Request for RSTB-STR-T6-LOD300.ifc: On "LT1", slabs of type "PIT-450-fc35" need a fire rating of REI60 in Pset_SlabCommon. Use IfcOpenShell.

First a look at what the model holds.

```python
import ifcopenshell
import ifcopenshell.util.element

model = ifcopenshell.open("RSTB-STR-T6-LOD300.ifc")
print(model.schema)
storey = next(s for s in model.by_type("IfcBuildingStorey") if s.Name == "LT1")
slabs = [e for e in ifcopenshell.util.element.get_decomposition(storey) if e.is_a("IfcSlab")]
seen = {}
for e in slabs:
    element_type = ifcopenshell.util.element.get_type(e)
    key = (element_type.Name if element_type != e and element_type else None, ifcopenshell.util.element.get_pset(e, "Pset_SlabCommon", "FireRating"))
    seen[key] = seen.get(key, 0) + 1
for (name, value), count in sorted(seen.items(), key=str):
    print(count, "x", name, "|", value)
```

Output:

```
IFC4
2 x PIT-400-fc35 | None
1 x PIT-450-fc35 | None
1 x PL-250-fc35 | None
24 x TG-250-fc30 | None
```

```python
import ifcopenshell
import ifcopenshell.api.pset
import ifcopenshell.util.element

model = ifcopenshell.open("RSTB-STR-T6-LOD300.ifc")

storey = next(s for s in model.by_type("IfcBuildingStorey") if s.Name == "LT1")
slabs = [e for e in ifcopenshell.util.element.get_decomposition(storey) if e.is_a("IfcSlab")]

count = 0
for e in slabs:
    element_type = ifcopenshell.util.element.get_type(e)
    if element_type in (None, e) or element_type.Name != "PIT-450-fc35":
        continue
    # add_pset returns the element's existing set when there is one.
    pset = ifcopenshell.api.pset.add_pset(model, product=e, name="Pset_SlabCommon")
    ifcopenshell.api.pset.edit_pset(model, pset=pset, properties={"FireRating": "REI60"})
    count += 1

print(count, "slabs updated")

model.write("RSTB-STR-T6-LOD300_updated.ifc")
```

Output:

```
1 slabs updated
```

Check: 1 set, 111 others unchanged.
